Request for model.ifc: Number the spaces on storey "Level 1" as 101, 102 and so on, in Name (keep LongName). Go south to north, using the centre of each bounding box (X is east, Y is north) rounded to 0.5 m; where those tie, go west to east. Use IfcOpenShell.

First a look at what the model holds.

```python
import ifcopenshell
import ifcopenshell.util.element
import ifcopenshell.util.placement

model = ifcopenshell.open("model.ifc")
print(model.schema)
storey = next(s for s in model.by_type("IfcBuildingStorey") if s.Name == "Level 1")
spaces = [e for e in ifcopenshell.util.element.get_decomposition(storey) if e.is_a("IfcSpace")]
for e in sorted(spaces, key=lambda e: e.id()):
    origin = ifcopenshell.util.placement.get_local_placement(e.ObjectPlacement)[:3, 3]
    print(e.id(), e.Name, e.LongName, origin.round(2) + 0.0, sep=" | ")
```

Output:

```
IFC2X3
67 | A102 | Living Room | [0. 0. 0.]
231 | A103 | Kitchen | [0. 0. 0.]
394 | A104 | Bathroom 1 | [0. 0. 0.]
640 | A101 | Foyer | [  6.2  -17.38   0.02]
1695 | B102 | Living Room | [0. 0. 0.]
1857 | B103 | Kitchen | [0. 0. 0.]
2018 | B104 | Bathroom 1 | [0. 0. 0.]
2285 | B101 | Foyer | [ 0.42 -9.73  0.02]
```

```python
import ifcopenshell
import ifcopenshell.geom
import ifcopenshell.util.element
import ifcopenshell.util.shape

model = ifcopenshell.open("model.ifc")
settings = ifcopenshell.geom.settings()
settings.set("use-world-coords", True)


def centre(element):
    shape = ifcopenshell.geom.create_shape(settings, element)
    return ifcopenshell.util.shape.get_bbox_centroid(shape.geometry)


storey = next(s for s in model.by_type("IfcBuildingStorey") if s.Name == "Level 1")
spaces = [e for e in ifcopenshell.util.element.get_decomposition(storey) if e.is_a("IfcSpace")]

# Insertion points can sit at a corner or the storey origin, so sort by the geometry (in metres).
centres = {e: centre(e) for e in spaces}
spaces.sort(key=lambda e: (round(centres[e][1] / 0.5), centres[e][0]))

for i, e in enumerate(spaces, start=1):
    number = f"1{i:02d}"
    e.Name = number
    print(e.id(), number)

model.write("model_edited.ifc")
```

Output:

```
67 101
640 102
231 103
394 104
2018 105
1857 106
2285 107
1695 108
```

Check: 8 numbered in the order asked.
